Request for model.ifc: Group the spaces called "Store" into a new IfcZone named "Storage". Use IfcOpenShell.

First a look at what the model holds.

```python
import ifcopenshell

model = ifcopenshell.open("model.ifc")
print(model.schema)
seen = {}
for space in model.by_type("IfcSpace"):
    seen[space.LongName] = seen.get(space.LongName, 0) + 1
for name, count in sorted(seen.items(), key=str):
    print(count, "x", name)
print("zones:", [z.Name for z in model.by_type("IfcZone")][:20])
```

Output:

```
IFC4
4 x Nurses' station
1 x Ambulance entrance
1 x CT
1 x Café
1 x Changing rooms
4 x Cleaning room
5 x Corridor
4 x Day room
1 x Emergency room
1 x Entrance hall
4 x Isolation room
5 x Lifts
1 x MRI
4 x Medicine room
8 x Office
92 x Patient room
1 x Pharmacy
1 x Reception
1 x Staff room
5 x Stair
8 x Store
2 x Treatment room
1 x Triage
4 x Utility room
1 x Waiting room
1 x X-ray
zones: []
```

```python
import ifcopenshell
import ifcopenshell.api.group
import ifcopenshell.api.root

model = ifcopenshell.open("model.ifc")

names = {"Store"}
spaces = [s for s in model.by_type("IfcSpace") if s.LongName in names]

zone = ifcopenshell.api.root.create_entity(model, ifc_class="IfcZone", name="Storage")
ifcopenshell.api.group.assign_group(model, products=spaces, group=zone)
print(len(spaces), "spaces in", zone.Name)

model.write("model_rev.ifc")
```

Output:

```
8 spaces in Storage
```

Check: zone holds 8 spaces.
